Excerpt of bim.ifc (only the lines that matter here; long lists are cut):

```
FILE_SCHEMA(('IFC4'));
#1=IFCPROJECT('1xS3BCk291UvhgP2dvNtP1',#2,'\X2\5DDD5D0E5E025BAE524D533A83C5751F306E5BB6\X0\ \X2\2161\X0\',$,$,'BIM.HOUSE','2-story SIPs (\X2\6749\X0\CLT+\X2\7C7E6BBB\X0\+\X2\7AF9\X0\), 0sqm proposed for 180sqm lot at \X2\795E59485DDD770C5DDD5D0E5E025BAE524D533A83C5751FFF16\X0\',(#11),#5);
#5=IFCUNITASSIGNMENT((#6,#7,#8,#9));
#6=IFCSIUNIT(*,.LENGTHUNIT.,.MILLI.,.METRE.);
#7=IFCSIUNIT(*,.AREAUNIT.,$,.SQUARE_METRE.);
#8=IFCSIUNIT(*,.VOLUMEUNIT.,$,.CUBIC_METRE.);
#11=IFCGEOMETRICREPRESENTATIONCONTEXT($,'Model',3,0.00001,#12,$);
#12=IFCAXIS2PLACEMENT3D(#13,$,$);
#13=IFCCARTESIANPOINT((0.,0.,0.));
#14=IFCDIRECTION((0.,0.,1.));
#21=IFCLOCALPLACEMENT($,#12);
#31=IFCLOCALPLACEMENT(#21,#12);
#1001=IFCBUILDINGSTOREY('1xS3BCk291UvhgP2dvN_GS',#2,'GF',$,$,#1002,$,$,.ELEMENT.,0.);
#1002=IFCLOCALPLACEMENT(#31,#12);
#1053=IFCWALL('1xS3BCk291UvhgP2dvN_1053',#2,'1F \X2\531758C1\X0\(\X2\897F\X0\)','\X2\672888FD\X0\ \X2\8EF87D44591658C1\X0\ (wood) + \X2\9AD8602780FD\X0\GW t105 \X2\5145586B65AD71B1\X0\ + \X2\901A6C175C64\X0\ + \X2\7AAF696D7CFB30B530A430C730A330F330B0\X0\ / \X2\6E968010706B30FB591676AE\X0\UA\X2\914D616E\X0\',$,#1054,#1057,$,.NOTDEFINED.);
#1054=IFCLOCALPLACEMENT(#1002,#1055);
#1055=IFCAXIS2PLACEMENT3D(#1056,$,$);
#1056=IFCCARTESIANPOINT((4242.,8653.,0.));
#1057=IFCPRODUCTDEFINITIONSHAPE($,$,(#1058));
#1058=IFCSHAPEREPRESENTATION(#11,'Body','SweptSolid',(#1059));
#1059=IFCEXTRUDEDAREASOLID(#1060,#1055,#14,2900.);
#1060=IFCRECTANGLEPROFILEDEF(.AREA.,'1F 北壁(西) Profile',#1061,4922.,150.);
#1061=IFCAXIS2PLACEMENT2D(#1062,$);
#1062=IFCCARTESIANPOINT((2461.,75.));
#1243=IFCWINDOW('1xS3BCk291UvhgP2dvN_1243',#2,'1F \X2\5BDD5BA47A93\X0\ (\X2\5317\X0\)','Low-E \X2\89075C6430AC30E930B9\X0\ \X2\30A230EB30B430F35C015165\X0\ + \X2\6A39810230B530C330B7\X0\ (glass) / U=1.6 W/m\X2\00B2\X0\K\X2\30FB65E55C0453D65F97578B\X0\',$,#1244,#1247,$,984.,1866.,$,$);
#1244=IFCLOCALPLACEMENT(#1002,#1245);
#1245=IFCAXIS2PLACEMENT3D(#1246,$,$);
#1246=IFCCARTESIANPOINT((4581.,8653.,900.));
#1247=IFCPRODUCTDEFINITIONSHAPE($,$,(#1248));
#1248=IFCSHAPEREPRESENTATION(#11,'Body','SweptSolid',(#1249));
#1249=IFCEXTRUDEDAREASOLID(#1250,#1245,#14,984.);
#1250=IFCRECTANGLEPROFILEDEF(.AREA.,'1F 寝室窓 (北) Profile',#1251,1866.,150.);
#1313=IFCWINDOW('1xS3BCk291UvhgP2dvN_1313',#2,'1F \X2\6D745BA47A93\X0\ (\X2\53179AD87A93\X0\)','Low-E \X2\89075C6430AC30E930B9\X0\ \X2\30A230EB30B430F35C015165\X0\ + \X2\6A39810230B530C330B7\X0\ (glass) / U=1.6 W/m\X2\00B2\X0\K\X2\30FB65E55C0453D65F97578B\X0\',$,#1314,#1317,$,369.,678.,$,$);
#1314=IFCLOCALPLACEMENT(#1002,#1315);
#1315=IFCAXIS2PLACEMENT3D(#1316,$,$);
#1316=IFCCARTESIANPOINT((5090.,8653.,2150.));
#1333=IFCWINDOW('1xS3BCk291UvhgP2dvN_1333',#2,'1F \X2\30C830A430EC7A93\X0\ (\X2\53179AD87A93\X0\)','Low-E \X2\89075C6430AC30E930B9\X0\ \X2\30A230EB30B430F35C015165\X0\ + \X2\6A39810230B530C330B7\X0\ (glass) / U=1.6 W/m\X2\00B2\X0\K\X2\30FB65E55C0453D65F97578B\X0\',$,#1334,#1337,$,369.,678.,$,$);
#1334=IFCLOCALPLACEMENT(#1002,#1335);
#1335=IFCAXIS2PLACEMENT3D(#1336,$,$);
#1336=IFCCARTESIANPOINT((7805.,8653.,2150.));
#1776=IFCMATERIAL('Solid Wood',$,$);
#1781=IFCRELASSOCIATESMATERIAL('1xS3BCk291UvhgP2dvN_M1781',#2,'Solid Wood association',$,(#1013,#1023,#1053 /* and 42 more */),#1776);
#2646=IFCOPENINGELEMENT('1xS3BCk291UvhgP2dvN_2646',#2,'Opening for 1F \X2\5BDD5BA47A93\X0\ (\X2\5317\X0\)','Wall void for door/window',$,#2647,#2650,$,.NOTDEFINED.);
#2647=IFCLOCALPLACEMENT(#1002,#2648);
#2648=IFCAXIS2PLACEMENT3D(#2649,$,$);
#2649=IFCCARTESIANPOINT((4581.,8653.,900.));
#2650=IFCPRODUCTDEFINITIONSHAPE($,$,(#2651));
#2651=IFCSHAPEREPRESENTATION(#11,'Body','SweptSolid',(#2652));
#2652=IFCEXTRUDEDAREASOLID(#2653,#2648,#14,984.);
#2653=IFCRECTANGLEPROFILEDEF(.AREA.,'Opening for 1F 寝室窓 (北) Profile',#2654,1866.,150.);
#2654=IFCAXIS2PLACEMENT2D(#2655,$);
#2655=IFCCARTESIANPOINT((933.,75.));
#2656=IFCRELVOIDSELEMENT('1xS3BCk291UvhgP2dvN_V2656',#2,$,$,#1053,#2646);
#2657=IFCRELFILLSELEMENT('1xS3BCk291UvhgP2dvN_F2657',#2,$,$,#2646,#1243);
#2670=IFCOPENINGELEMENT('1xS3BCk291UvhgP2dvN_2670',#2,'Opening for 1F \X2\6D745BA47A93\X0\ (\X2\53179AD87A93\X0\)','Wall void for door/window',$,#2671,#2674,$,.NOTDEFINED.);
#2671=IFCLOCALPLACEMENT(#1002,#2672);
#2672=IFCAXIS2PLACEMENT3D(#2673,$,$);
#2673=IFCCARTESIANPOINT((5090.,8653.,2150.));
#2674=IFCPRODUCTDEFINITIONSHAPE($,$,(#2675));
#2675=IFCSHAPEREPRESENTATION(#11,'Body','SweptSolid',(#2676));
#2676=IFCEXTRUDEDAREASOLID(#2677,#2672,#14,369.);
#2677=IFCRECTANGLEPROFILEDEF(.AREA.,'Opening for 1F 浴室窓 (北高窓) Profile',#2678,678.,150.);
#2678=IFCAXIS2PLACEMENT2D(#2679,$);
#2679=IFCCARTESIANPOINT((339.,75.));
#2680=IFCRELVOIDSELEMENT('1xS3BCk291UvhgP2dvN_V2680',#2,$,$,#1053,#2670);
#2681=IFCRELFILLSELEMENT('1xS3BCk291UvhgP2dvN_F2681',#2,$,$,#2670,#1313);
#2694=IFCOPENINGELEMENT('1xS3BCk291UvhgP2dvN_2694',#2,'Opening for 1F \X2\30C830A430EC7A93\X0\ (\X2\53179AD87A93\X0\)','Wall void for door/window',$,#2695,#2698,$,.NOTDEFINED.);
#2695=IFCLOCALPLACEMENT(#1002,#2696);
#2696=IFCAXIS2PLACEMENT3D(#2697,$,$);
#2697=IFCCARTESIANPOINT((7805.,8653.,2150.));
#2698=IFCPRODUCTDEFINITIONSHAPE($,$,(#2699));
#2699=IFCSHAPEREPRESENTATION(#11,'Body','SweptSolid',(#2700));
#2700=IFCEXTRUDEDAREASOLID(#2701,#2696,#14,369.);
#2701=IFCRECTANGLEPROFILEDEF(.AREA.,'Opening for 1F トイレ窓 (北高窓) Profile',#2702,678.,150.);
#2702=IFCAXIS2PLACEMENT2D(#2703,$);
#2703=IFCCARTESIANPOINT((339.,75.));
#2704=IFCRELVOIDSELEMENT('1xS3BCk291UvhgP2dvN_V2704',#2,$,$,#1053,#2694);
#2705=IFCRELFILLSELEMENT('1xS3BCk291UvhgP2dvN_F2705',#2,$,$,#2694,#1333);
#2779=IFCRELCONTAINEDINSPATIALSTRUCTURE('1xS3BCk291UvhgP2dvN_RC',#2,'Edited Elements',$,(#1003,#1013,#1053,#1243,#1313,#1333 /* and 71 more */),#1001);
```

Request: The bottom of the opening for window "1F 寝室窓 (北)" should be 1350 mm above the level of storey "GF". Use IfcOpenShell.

```python
import numpy as np
import ifcopenshell
import ifcopenshell.api.geometry
import ifcopenshell.geom
import ifcopenshell.util.element
import ifcopenshell.util.placement
import ifcopenshell.util.shape
import ifcopenshell.util.unit

model = ifcopenshell.open("bim.ifc")
unit_scale = ifcopenshell.util.unit.calculate_unit_scale(model)

window = model.by_id(1243)
opening = window.FillsVoids[0].RelatingOpeningElement
storey = ifcopenshell.util.element.get_container(window, ifc_class="IfcBuildingStorey")
level = ifcopenshell.util.placement.get_local_placement(storey.ObjectPlacement)[2, 3]

# The opening's origin need not be at the sill, so measure its lowest point.
shape = ifcopenshell.geom.create_shape(ifcopenshell.geom.settings(), opening)
bottom = ifcopenshell.util.shape.get_shape_bottom_elevation(shape, shape.geometry) / unit_scale
dz = level + 1.35 / unit_scale - bottom

shift = np.array([0.0, 0.0, dz])
# The window is not placed relative to its opening, so move both.
for product in (opening, window):
    matrix = ifcopenshell.util.placement.get_local_placement(product.ObjectPlacement)
    matrix[:3, 3] += shift
    ifcopenshell.api.geometry.edit_object_placement(model, product=product, matrix=matrix, is_si=False)

print(f"moved by {dz * unit_scale:+.3f} m")

model.write("bim_v2.ifc")
```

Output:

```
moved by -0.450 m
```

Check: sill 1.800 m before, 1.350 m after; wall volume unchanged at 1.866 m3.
